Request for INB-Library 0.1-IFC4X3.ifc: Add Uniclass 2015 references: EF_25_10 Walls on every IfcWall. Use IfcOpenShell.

First a look at what the model holds.

```python
import ifcopenshell

model = ifcopenshell.open("INB-Library 0.1-IFC4X3.ifc")
print(model.schema)
print("classifications:", [c.Name for c in model.by_type("IfcClassification")])
for ifc_class in ("IfcDoor", "IfcRoof", "IfcStair", "IfcWall", "IfcWindow"):
    print(ifc_class, len(model.by_type(ifc_class)))
```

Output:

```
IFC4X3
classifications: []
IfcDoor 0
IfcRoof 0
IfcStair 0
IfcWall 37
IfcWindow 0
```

```python
import ifcopenshell
import ifcopenshell.api.classification

model = ifcopenshell.open("INB-Library 0.1-IFC4X3.ifc")

system = ifcopenshell.api.classification.add_classification(model, classification="Uniclass 2015")

codes = {
    "IfcWall": ("EF_25_10", "Walls"),
}
for ifc_class, (code, name) in codes.items():
    products = model.by_type(ifc_class)
    ifcopenshell.api.classification.add_reference(
        model, products=products, classification=system, identification=code, name=name
    )
    print(code, len(products))

model.write("INB-Library 0.1-IFC4X3_rev.ifc")
```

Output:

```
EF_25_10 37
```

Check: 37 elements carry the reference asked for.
